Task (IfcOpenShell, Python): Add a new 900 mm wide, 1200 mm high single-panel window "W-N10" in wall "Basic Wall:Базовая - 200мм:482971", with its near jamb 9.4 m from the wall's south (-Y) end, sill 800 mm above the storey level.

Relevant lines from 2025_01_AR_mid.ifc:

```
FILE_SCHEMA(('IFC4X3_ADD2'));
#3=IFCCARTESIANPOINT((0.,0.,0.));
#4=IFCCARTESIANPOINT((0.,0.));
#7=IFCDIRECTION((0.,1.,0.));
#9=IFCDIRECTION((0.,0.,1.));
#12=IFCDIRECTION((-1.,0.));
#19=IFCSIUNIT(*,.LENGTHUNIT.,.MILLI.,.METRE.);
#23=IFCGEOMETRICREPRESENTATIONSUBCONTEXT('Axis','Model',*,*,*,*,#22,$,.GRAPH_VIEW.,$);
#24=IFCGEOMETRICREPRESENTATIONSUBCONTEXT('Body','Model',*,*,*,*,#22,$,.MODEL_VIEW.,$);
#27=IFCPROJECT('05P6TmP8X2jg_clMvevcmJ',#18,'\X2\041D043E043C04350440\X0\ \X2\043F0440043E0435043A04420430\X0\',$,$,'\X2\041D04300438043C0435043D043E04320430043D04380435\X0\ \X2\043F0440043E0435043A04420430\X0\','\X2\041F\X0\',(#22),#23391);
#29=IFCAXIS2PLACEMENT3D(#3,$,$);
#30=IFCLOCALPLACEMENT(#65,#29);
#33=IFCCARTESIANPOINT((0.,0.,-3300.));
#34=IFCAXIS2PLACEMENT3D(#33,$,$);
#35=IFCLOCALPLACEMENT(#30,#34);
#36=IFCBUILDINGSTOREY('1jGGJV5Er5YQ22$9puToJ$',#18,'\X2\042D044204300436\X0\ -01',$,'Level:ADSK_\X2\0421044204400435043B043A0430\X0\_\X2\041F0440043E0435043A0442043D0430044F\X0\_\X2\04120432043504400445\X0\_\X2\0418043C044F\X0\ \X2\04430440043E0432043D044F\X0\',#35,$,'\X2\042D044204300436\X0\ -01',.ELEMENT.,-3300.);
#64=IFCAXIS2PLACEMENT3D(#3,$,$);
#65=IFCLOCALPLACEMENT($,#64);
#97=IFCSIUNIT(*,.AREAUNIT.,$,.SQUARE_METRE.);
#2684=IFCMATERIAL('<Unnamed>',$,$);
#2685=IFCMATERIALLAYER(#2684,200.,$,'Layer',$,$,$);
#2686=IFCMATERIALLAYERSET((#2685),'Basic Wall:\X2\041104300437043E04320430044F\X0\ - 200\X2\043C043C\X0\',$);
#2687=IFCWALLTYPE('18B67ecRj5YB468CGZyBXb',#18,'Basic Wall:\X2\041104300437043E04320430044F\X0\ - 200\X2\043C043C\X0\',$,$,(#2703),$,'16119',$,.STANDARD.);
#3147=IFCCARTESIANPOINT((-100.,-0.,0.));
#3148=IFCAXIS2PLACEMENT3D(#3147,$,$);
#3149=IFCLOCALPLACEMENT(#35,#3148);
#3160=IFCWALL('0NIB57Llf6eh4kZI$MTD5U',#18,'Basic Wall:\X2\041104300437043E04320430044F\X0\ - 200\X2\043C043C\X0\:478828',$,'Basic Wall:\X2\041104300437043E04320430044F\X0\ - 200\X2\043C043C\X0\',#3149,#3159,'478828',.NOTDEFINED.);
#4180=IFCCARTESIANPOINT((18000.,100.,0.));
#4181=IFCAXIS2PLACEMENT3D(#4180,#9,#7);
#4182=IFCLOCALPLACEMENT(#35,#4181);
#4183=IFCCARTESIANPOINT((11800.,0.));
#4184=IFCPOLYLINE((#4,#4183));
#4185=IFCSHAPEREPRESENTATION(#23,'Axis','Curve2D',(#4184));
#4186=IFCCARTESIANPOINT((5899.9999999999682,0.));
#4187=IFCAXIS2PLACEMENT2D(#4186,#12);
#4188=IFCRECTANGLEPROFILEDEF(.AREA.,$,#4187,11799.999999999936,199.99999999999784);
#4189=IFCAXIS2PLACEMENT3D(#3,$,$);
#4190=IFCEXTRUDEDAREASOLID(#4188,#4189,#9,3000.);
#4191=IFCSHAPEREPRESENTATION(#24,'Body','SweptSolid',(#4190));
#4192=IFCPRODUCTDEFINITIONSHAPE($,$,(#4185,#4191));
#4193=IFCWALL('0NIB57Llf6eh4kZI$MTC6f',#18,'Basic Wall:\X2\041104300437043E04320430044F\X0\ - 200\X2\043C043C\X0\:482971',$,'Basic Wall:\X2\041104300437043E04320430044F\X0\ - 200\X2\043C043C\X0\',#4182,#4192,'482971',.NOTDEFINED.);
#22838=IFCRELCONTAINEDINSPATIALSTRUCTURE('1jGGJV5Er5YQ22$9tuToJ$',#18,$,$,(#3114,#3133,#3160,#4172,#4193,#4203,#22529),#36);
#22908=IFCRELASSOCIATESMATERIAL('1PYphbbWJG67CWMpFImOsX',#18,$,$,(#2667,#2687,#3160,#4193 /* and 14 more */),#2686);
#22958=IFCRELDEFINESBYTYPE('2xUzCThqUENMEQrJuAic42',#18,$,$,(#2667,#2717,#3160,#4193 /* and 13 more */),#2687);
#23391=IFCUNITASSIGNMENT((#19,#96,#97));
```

```python
import numpy as np
import ifcopenshell
import ifcopenshell.api.feature
import ifcopenshell.api.geometry
import ifcopenshell.api.root
import ifcopenshell.api.spatial
import ifcopenshell.geom
import ifcopenshell.util.element
import ifcopenshell.util.placement
import ifcopenshell.util.representation
import ifcopenshell.util.shape
import ifcopenshell.util.unit

model = ifcopenshell.open("2025_01_AR_mid.ifc")
unit_scale = ifcopenshell.util.unit.calculate_unit_scale(model)
settings = ifcopenshell.geom.settings()


def volume(element):
    """Net volume in cubic metres, openings subtracted."""
    shape = ifcopenshell.geom.create_shape(settings, element)
    return ifcopenshell.util.shape.get_volume(shape.geometry)


wall = model.by_guid("0NIB57Llf6eh4kZI$MTC6f")
storey = ifcopenshell.util.element.get_container(wall, ifc_class="IfcBuildingStorey")
context = ifcopenshell.util.representation.get_context(model, "Model", "Body", "MODEL_VIEW")
before = volume(wall)

width, height, from_end, sill = 0.9, 1.2, 9.4, 0.8  # metres

# The wall runs along its own X axis, and the end named is its -X end.
wall_shape = ifcopenshell.geom.create_shape(settings, wall)
x, y, z = ifcopenshell.util.shape.get_vertices(wall_shape.geometry).T
start = x.min() + from_end
face, thickness = float(y.min()), float(y.max() - y.min())
wall_matrix = ifcopenshell.util.placement.get_local_placement(wall.ObjectPlacement)
level = ifcopenshell.util.placement.get_local_placement(storey.ObjectPlacement)[2, 3]


def in_wall(x, y):
    """Placement at x, y metres in the wall's axes, at sill height."""
    matrix = wall_matrix.copy()
    matrix[:, 3] = wall_matrix @ np.array([x / unit_scale, y / unit_scale, 0.0, 1.0])
    matrix[2, 3] = level + sill / unit_scale
    return matrix


# Opening: a box that overshoots both wall faces by 50 mm.
opening = ifcopenshell.api.root.create_entity(model, ifc_class="IfcOpeningElement", predefined_type="OPENING")
box = ifcopenshell.api.geometry.add_wall_representation(
    model, context=context, length=width, height=height, thickness=thickness + 0.1
)
ifcopenshell.api.geometry.assign_representation(model, product=opening, representation=box)
ifcopenshell.api.geometry.edit_object_placement(model, product=opening, matrix=in_wall(start, face - 0.05), is_si=False)
ifcopenshell.api.feature.add_feature(model, feature=opening, element=wall)

window = ifcopenshell.api.root.create_entity(model, ifc_class="IfcWindow", name="W-N10", predefined_type="WINDOW")
window.OverallWidth, window.OverallHeight = width / unit_scale, height / unit_scale
window.PartitioningType = "SINGLE_PANEL"
body = ifcopenshell.api.geometry.add_window_representation(
    model,
    context=context,
    overall_width=window.OverallWidth,
    overall_height=window.OverallHeight,
    partition_type="SINGLE_PANEL",
)
ifcopenshell.api.geometry.assign_representation(model, product=window, representation=body)
ifcopenshell.api.spatial.assign_container(model, products=[window], relating_structure=storey)
ifcopenshell.api.feature.add_filling(model, opening=opening, element=window)

# Centre the window in the wall's thickness.
ifcopenshell.api.geometry.edit_object_placement(model, product=window, matrix=in_wall(start, face), is_si=False)
window_shape = ifcopenshell.geom.create_shape(settings, window)
depth = ifcopenshell.util.shape.get_vertices(window_shape.geometry)[:, 1]
offset = face + thickness / 2 - (depth.min() + depth.max()) / 2
ifcopenshell.api.geometry.edit_object_placement(model, product=window, matrix=in_wall(start, offset), is_si=False)

after = volume(wall)

print(f"wall volume {before:.3f} -> {after:.3f} m3")

model.write("2025_01_AR_mid_rev.ifc")
```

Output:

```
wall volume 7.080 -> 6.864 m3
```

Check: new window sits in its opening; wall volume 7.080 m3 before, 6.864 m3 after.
